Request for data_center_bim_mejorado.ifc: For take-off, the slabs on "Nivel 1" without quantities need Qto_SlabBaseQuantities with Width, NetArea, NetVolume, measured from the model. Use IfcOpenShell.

First a look at what the model holds.

```python
import ifcopenshell
import ifcopenshell.util.element
import ifcopenshell.util.unit

model = ifcopenshell.open("data_center_bim_mejorado.ifc")
print(model.schema)
for unit_type in ("LENGTHUNIT", "AREAUNIT", "VOLUMEUNIT"):
    print(unit_type, ifcopenshell.util.unit.calculate_unit_scale(model, unit_type))
storey = next(s for s in model.by_type("IfcBuildingStorey") if s.Name == "Nivel 1")
slabs = [e for e in ifcopenshell.util.element.get_decomposition(storey) if e.is_a("IfcSlab")]
for e in sorted(slabs, key=lambda e: e.id()):
    print(e.id(), e.is_a(), e.Name, list(ifcopenshell.util.element.get_psets(e, qtos_only=True)), sep=" | ")
```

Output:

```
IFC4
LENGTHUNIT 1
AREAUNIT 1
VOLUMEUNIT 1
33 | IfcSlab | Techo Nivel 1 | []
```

```python
import ifcopenshell
import ifcopenshell.api.pset
import ifcopenshell.geom
import ifcopenshell.util.element
import ifcopenshell.util.shape
import ifcopenshell.util.unit

model = ifcopenshell.open("data_center_bim_mejorado.ifc")
unit_scale = ifcopenshell.util.unit.calculate_unit_scale(model)
area_scale = ifcopenshell.util.unit.calculate_unit_scale(model, "AREAUNIT")
volume_scale = ifcopenshell.util.unit.calculate_unit_scale(model, "VOLUMEUNIT")
settings = ifcopenshell.geom.settings()

storey = next(s for s in model.by_type("IfcBuildingStorey") if s.Name == "Nivel 1")
slabs = [e for e in ifcopenshell.util.element.get_decomposition(storey) if e.is_a("IfcSlab")]

for e in sorted(slabs, key=lambda e: e.id()):
    if ifcopenshell.util.element.get_psets(e, qtos_only=True, should_inherit=False):
        continue
    # Geometry comes back in metres, in the element's own axes.
    shape = ifcopenshell.geom.create_shape(settings, e)
    values = {
        "Width": ifcopenshell.util.shape.get_z(shape.geometry) / unit_scale,
        "NetArea": ifcopenshell.util.shape.get_footprint_area(shape.geometry) / area_scale,
        "NetVolume": ifcopenshell.util.shape.get_volume(shape.geometry) / volume_scale,
    }
    qto = ifcopenshell.api.pset.add_qto(model, product=e, name="Qto_SlabBaseQuantities")
    ifcopenshell.api.pset.edit_qto(model, qto=qto, properties=values)
    print(e.id(), {k: round(v, 3) for k, v in values.items()})

model.write("data_center_bim_mejorado_updated.ifc")
```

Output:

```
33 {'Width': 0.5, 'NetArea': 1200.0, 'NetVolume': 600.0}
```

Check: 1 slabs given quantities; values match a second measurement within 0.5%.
